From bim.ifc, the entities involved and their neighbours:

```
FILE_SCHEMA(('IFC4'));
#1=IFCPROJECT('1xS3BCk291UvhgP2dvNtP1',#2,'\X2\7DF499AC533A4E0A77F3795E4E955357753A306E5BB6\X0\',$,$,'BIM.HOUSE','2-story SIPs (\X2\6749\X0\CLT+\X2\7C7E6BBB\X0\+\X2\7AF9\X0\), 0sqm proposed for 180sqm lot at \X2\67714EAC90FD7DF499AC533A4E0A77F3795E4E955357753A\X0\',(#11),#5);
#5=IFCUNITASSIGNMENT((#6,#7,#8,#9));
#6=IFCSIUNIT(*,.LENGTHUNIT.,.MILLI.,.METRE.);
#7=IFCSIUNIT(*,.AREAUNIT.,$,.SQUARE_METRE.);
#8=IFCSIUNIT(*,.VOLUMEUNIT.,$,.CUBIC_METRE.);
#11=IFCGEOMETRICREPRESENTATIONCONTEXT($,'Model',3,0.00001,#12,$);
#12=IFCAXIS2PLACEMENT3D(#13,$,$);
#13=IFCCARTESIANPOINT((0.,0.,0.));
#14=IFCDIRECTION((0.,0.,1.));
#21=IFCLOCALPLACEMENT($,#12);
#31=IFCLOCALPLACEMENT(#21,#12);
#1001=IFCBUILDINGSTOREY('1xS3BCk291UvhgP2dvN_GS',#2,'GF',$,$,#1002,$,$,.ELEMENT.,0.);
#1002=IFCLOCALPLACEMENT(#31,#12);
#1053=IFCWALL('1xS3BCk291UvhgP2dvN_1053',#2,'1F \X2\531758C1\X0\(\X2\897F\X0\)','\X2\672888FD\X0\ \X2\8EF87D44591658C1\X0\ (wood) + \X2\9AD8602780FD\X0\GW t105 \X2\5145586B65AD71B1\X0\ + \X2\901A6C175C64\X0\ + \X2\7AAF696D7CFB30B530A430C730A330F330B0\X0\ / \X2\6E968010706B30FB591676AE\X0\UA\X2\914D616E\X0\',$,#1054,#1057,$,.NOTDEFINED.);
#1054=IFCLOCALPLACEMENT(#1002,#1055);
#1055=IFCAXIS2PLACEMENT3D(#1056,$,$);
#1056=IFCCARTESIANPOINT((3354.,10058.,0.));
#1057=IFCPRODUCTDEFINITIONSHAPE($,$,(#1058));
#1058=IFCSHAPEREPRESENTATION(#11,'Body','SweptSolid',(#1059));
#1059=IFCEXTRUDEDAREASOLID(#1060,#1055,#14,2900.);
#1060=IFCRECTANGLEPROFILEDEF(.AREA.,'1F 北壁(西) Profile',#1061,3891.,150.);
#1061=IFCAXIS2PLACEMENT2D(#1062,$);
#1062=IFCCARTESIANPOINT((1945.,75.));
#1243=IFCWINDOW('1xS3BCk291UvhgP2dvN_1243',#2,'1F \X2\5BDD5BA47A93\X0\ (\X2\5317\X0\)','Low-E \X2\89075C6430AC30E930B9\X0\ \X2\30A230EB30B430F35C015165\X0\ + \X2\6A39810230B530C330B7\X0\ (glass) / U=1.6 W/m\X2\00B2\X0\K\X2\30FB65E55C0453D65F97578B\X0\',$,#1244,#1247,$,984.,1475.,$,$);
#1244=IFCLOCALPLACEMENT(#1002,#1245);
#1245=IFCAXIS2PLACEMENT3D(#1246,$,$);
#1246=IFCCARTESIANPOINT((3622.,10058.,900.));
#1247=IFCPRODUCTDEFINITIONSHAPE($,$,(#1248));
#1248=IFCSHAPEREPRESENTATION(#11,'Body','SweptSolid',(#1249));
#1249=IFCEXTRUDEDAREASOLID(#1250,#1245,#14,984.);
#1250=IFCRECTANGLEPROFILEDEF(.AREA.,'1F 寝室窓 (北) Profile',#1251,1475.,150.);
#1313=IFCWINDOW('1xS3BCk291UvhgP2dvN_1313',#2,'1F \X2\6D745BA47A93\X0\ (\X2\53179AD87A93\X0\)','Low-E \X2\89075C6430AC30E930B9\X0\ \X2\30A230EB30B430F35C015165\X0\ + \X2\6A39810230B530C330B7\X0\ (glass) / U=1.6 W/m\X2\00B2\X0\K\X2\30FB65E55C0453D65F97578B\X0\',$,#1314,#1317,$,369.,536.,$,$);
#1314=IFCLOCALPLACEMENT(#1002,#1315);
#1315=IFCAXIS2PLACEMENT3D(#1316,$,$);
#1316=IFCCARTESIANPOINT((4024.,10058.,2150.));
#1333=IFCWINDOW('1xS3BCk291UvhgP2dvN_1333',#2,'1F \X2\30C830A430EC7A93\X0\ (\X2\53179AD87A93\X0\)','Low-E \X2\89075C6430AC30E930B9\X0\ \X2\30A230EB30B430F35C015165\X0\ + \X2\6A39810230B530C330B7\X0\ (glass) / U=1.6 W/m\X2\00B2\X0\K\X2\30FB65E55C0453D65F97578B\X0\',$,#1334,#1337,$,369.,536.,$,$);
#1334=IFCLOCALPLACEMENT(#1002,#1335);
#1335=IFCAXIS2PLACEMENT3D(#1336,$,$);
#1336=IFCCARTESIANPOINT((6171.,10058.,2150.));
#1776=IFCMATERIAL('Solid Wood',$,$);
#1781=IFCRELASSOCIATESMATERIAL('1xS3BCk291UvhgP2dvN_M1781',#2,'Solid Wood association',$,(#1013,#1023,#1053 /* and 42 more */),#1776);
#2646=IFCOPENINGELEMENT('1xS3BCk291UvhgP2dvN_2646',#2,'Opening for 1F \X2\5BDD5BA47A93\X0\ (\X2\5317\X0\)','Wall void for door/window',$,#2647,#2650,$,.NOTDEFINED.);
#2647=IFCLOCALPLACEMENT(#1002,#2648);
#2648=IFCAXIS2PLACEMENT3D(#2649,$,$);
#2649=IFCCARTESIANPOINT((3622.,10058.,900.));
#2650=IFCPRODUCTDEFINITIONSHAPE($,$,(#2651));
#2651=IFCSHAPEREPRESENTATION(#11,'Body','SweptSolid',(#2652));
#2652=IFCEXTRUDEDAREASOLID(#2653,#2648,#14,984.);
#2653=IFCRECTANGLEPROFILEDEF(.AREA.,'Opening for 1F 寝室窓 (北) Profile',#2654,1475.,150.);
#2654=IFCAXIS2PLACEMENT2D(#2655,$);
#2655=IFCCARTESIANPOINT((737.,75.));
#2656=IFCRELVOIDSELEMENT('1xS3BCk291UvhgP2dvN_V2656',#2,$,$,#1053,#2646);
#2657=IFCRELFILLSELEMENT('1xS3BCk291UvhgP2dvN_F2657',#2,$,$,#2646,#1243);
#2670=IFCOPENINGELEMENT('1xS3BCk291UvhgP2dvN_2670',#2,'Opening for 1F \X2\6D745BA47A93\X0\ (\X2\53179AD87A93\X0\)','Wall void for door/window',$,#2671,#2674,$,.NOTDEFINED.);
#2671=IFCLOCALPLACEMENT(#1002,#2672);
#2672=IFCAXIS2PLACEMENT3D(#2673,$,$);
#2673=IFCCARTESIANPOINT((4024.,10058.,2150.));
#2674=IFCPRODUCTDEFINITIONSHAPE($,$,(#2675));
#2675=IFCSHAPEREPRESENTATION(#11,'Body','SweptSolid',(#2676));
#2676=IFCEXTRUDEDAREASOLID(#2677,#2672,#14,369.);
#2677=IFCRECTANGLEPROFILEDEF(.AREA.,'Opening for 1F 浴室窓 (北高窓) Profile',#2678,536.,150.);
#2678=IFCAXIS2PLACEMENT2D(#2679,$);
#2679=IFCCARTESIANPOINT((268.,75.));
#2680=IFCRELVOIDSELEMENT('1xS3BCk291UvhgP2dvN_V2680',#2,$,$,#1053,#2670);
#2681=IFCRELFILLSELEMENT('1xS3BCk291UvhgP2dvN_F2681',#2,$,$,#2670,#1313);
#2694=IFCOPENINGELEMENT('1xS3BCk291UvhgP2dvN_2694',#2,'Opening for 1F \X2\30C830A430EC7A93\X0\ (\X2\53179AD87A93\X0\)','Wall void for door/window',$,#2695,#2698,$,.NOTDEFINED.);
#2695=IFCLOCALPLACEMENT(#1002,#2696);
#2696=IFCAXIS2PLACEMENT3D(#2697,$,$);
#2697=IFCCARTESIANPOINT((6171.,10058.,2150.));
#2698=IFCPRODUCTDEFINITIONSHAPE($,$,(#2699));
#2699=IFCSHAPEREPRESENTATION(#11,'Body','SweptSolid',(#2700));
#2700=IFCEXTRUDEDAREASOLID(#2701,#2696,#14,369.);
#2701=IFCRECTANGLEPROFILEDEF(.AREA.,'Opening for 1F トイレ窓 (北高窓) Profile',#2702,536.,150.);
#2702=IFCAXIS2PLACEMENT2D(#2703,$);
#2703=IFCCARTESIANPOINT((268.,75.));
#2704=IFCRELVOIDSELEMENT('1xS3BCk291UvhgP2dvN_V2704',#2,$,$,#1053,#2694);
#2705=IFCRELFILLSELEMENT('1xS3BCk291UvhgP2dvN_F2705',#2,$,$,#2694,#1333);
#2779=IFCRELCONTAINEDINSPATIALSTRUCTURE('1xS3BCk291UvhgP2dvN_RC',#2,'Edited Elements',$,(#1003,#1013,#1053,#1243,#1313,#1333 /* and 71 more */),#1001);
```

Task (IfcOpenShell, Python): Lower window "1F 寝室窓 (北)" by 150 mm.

```python
import numpy as np
import ifcopenshell
import ifcopenshell.api.geometry
import ifcopenshell.util.placement
import ifcopenshell.util.unit

model = ifcopenshell.open("bim.ifc")
unit_scale = ifcopenshell.util.unit.calculate_unit_scale(model)

window = model.by_id(1243)
opening = window.FillsVoids[0].RelatingOpeningElement
dz = -0.15 / unit_scale

shift = np.array([0.0, 0.0, dz])
# The window is not placed relative to its opening, so move both.
for product in (opening, window):
    matrix = ifcopenshell.util.placement.get_local_placement(product.ObjectPlacement)
    matrix[:3, 3] += shift
    ifcopenshell.api.geometry.edit_object_placement(model, product=product, matrix=matrix, is_si=False)

print(f"moved by {dz * unit_scale:+.3f} m")

model.write("bim_rev.ifc")
```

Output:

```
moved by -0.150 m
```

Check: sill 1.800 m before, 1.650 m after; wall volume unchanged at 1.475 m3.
